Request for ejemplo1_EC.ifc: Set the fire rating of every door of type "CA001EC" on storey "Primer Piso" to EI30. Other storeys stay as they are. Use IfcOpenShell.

First a look at what the model holds.

```python
import ifcopenshell
import ifcopenshell.util.element

model = ifcopenshell.open("ejemplo1_EC.ifc")
print(model.schema)
storey = next(s for s in model.by_type("IfcBuildingStorey") if s.Name == "Primer Piso")
doors = [e for e in ifcopenshell.util.element.get_decomposition(storey) if e.is_a("IfcDoor")]
seen = {}
for e in doors:
    element_type = ifcopenshell.util.element.get_type(e)
    key = (element_type.Name if element_type != e and element_type else None, ifcopenshell.util.element.get_pset(e, "Pset_DoorCommon", "FireRating"))
    seen[key] = seen.get(key, 0) + 1
for (name, value), count in sorted(seen.items(), key=str):
    print(count, "x", name, "|", value)
```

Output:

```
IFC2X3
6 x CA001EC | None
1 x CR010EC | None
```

```python
import ifcopenshell
import ifcopenshell.api.pset
import ifcopenshell.util.element

model = ifcopenshell.open("ejemplo1_EC.ifc")

storey = next(s for s in model.by_type("IfcBuildingStorey") if s.Name == "Primer Piso")
doors = [e for e in ifcopenshell.util.element.get_decomposition(storey) if e.is_a("IfcDoor")]

count = 0
for e in doors:
    element_type = ifcopenshell.util.element.get_type(e)
    if element_type in (None, e) or element_type.Name != "CA001EC":
        continue
    # add_pset returns the element's existing set when there is one.
    pset = ifcopenshell.api.pset.add_pset(model, product=e, name="Pset_DoorCommon")
    ifcopenshell.api.pset.edit_pset(model, pset=pset, properties={"FireRating": "EI30"})
    count += 1

print(count, "doors updated")

model.write("ejemplo1_EC-out.ifc")
```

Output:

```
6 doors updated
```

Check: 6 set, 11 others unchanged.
